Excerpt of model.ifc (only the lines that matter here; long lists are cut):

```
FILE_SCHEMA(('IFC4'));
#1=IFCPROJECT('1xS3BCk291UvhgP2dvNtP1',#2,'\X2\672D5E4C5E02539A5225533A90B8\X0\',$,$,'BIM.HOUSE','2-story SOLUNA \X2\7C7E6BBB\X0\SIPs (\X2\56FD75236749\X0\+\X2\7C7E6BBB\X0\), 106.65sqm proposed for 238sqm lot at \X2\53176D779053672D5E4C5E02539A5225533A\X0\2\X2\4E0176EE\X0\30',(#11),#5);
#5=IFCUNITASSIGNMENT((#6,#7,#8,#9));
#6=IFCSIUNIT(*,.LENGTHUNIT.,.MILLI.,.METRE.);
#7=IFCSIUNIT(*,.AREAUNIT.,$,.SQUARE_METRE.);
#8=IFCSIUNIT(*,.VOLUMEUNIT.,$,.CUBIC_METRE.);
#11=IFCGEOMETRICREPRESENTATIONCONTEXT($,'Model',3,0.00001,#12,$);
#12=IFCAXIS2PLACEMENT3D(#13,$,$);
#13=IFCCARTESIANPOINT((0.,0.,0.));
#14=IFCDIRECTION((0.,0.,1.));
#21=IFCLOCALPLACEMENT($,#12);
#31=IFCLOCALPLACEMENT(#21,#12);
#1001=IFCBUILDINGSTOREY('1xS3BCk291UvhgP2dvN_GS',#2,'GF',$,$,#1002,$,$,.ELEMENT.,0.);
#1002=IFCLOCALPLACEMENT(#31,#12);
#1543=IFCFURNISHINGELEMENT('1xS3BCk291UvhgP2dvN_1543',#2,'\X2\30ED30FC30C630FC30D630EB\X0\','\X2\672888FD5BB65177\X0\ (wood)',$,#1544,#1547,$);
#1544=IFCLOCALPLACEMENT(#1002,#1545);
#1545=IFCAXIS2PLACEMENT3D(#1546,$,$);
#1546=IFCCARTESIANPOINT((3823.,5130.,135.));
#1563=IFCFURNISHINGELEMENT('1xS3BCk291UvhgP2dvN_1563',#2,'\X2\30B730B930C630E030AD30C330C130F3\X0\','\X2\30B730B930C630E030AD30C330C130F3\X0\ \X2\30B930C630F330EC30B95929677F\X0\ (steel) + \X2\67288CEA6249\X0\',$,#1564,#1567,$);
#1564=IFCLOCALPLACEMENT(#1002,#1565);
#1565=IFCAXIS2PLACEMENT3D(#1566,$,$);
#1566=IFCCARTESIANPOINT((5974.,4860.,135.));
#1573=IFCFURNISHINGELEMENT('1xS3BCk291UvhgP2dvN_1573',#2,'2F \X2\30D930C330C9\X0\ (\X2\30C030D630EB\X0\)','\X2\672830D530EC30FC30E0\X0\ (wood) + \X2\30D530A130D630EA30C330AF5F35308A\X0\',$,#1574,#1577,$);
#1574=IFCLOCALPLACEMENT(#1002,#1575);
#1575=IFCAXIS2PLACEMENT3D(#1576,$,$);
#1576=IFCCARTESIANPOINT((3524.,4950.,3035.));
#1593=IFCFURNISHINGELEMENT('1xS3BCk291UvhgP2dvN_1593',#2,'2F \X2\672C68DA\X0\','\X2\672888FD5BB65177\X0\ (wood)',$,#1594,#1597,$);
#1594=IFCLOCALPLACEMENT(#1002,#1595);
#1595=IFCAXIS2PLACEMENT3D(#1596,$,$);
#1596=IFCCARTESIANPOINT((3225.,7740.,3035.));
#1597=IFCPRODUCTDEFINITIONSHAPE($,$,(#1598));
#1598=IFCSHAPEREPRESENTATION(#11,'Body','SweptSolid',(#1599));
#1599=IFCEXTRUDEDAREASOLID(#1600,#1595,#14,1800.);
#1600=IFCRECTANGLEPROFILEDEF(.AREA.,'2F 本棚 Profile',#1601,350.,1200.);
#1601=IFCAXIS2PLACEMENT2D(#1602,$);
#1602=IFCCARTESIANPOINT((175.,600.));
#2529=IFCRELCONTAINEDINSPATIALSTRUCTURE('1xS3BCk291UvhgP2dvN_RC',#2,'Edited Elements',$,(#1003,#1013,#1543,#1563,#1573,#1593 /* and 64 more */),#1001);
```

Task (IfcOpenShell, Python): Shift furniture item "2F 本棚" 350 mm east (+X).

```python
import ifcopenshell
import ifcopenshell.api.geometry
import ifcopenshell.util.placement

model = ifcopenshell.open("model.ifc")

item = model.by_guid("1xS3BCk291UvhgP2dvN_1593")
matrix = ifcopenshell.util.placement.get_local_placement(item.ObjectPlacement)
matrix[0, 3] += 350.0
ifcopenshell.api.geometry.edit_object_placement(model, product=item, matrix=matrix, is_si=False)

print(ifcopenshell.util.placement.get_local_placement(item.ObjectPlacement).round(3) + 0.0)

model.write("model_rev.ifc")
```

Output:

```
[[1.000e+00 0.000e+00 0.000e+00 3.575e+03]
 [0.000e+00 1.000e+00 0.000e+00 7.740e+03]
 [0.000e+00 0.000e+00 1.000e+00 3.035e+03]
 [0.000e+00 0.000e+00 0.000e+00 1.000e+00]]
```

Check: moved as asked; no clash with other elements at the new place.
